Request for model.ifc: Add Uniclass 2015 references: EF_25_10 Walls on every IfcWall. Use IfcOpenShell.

First a look at what the model holds.

```python
import ifcopenshell

model = ifcopenshell.open("model.ifc")
print(model.schema)
print("classifications:", [c.Name for c in model.by_type("IfcClassification")])
for ifc_class in ("IfcDoor", "IfcRoof", "IfcStair", "IfcWall", "IfcWindow"):
    print(ifc_class, len(model.by_type(ifc_class)))
```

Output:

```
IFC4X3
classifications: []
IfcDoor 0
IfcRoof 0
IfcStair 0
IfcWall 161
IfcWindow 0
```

```python
import ifcopenshell
import ifcopenshell.api.classification

model = ifcopenshell.open("model.ifc")

system = ifcopenshell.api.classification.add_classification(model, classification="Uniclass 2015")

codes = {
    "IfcWall": ("EF_25_10", "Walls"),
}
for ifc_class, (code, name) in codes.items():
    products = model.by_type(ifc_class)
    ifcopenshell.api.classification.add_reference(
        model, products=products, classification=system, identification=code, name=name
    )
    print(code, len(products))

model.write("model_updated.ifc")
```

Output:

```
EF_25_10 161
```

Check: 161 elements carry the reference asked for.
